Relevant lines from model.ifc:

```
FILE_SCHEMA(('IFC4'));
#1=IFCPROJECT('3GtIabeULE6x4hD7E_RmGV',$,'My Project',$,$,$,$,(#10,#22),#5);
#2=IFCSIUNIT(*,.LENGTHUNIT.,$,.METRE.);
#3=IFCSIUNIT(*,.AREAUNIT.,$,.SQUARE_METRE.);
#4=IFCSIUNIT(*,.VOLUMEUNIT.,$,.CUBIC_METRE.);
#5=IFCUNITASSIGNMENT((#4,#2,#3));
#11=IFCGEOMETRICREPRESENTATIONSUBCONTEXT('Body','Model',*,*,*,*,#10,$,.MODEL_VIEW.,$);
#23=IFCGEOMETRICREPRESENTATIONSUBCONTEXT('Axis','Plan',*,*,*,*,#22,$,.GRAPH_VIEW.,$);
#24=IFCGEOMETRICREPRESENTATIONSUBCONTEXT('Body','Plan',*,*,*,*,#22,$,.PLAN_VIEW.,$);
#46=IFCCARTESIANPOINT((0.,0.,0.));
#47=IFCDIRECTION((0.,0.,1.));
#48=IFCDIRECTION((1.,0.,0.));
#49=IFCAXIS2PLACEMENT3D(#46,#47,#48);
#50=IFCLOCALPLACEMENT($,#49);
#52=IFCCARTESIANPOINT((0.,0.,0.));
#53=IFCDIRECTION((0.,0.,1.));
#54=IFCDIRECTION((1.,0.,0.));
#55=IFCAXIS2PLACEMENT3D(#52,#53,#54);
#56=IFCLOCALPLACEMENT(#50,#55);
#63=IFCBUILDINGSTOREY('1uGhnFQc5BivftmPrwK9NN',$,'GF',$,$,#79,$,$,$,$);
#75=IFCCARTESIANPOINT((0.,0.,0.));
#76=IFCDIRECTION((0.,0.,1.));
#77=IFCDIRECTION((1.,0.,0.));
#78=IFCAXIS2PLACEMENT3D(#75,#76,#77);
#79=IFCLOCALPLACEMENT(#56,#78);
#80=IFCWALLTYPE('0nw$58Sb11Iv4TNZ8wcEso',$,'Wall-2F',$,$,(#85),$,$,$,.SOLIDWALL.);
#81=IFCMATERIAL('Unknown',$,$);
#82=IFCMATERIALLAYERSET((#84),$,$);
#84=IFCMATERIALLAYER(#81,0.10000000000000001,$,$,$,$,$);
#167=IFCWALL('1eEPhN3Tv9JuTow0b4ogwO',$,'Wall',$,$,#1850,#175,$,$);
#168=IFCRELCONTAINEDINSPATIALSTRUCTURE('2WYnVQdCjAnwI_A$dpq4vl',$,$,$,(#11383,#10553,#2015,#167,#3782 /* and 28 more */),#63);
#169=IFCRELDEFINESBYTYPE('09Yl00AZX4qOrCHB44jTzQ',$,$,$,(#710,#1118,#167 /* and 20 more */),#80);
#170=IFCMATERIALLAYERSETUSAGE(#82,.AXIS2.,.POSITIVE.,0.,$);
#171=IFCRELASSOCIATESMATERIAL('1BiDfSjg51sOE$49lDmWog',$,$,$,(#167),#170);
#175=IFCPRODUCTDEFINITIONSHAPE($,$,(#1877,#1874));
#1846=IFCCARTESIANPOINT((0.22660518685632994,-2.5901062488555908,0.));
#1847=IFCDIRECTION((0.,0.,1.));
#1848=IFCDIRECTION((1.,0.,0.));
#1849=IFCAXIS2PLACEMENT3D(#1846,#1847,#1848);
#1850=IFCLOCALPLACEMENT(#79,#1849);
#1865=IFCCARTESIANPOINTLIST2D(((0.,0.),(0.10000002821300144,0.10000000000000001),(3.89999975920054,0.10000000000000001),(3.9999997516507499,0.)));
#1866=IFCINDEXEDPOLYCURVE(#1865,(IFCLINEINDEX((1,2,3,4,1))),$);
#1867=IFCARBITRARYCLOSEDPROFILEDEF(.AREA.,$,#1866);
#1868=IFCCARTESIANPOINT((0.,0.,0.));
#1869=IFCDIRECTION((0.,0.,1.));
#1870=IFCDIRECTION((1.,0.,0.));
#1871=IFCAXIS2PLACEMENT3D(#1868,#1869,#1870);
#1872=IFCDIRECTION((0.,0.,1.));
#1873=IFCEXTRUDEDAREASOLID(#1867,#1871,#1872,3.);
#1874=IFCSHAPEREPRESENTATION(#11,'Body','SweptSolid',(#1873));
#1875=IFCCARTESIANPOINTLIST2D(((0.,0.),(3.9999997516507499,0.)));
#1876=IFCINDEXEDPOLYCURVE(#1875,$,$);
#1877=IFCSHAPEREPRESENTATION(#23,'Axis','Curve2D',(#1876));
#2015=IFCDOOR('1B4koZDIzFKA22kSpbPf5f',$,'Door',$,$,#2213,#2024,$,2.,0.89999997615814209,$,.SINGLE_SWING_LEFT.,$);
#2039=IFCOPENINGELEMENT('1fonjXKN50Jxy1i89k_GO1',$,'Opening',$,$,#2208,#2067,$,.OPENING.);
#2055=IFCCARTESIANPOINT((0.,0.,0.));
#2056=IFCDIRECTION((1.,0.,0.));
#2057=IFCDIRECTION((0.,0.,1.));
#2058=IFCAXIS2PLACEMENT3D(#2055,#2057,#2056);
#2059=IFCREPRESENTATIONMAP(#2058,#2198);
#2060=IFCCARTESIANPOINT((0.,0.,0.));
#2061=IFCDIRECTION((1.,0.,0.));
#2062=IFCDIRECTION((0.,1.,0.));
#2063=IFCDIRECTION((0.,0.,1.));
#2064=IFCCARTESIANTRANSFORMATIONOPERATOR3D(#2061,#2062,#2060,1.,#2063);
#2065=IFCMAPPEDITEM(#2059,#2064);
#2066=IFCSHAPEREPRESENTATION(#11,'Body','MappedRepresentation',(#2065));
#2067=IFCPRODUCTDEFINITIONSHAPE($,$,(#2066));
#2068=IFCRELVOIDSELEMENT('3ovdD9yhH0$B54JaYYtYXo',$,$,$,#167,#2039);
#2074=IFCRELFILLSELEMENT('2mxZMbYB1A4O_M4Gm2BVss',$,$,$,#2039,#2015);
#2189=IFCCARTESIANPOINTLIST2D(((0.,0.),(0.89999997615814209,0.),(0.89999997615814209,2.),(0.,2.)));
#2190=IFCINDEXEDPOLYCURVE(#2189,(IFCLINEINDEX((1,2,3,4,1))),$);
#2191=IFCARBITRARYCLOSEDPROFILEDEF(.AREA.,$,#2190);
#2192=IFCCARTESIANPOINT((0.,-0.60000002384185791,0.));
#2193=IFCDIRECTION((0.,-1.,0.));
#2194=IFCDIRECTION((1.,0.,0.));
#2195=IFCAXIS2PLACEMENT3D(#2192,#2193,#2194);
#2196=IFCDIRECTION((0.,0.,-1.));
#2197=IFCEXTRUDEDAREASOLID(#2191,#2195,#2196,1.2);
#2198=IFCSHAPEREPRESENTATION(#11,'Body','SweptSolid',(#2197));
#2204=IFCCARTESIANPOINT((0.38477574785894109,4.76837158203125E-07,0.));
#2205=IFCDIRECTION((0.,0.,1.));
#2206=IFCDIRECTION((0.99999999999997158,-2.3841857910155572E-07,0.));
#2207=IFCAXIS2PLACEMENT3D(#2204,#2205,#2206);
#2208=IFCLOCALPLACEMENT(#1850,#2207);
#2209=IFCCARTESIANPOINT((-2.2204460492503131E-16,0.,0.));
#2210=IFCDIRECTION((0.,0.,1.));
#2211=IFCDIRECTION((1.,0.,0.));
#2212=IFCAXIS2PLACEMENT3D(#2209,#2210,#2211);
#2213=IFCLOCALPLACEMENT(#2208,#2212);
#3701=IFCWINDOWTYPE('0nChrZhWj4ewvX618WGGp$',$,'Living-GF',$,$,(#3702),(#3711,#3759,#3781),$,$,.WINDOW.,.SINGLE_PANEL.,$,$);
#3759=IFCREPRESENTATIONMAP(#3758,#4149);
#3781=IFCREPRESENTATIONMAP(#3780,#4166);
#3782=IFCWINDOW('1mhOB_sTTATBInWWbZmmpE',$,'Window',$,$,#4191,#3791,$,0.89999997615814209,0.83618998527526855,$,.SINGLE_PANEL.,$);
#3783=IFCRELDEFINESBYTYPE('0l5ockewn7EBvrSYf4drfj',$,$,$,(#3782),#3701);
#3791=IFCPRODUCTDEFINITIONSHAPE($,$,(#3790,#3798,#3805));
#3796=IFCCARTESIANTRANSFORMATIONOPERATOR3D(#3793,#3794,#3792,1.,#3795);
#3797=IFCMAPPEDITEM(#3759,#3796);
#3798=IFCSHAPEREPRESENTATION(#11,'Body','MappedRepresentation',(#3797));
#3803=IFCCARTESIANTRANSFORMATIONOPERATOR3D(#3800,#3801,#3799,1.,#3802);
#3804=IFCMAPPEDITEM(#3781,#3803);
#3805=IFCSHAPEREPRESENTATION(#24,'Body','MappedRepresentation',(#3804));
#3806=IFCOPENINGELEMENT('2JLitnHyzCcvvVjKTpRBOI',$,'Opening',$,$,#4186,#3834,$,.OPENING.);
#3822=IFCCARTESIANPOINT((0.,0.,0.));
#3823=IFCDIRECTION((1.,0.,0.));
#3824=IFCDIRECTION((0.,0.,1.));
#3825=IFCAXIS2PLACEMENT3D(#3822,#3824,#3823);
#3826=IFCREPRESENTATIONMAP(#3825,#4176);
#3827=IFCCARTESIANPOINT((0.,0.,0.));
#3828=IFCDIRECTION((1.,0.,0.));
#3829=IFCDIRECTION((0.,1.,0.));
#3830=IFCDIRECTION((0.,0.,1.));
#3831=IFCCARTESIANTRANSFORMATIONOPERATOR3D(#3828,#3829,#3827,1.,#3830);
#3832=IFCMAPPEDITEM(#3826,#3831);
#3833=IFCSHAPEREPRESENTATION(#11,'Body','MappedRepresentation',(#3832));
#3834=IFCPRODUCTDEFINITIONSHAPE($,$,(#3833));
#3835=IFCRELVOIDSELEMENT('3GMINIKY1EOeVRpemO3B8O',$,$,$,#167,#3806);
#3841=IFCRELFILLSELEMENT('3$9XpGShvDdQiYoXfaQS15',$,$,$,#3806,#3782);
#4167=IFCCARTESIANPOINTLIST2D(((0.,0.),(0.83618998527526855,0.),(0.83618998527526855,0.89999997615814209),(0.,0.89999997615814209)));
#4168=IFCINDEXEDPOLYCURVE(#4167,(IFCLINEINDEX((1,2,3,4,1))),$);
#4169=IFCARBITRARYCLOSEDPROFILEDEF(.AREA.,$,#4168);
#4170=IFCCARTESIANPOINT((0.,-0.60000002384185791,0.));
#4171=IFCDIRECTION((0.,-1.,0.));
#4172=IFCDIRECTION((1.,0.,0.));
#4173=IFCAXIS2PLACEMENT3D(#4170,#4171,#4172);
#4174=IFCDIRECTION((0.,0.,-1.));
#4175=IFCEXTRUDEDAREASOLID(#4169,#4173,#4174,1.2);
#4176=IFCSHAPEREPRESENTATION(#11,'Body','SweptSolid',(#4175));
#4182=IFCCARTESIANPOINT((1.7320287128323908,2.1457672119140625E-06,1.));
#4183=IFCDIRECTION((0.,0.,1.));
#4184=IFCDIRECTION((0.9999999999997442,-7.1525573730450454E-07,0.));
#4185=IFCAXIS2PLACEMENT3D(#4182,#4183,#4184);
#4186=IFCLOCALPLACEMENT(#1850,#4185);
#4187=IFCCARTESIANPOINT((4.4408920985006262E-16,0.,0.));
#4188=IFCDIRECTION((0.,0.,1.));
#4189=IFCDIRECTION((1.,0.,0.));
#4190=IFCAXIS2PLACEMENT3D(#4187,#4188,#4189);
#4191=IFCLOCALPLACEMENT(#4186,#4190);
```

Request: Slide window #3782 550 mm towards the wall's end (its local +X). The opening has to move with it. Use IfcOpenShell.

```python
import ifcopenshell
import ifcopenshell.api.geometry
import ifcopenshell.util.placement
import ifcopenshell.util.unit

model = ifcopenshell.open("model.ifc")
unit_scale = ifcopenshell.util.unit.calculate_unit_scale(model)

window = model.by_guid("1mhOB_sTTATBInWWbZmmpE")
opening = window.FillsVoids[0].RelatingOpeningElement
wall = opening.VoidsElements[0].RelatingBuildingElement

wall_matrix = ifcopenshell.util.placement.get_local_placement(wall.ObjectPlacement)
shift = wall_matrix[:3, 0] * 0.55 / unit_scale
before = ifcopenshell.util.placement.get_local_placement(window.ObjectPlacement)[:3, 3].copy()

# The window is placed relative to its opening, so it follows when the opening moves.
matrix = ifcopenshell.util.placement.get_local_placement(opening.ObjectPlacement)
matrix[:3, 3] += shift
ifcopenshell.api.geometry.edit_object_placement(
    model, product=opening, matrix=matrix, is_si=False, should_transform_children=True
)

after = ifcopenshell.util.placement.get_local_placement(window.ObjectPlacement)[:3, 3]
print("window moved by", (after - before).round(3) + 0.0)

model.write("model-out.ifc")
```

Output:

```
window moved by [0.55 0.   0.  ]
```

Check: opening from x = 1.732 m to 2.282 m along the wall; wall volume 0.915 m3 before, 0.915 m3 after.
